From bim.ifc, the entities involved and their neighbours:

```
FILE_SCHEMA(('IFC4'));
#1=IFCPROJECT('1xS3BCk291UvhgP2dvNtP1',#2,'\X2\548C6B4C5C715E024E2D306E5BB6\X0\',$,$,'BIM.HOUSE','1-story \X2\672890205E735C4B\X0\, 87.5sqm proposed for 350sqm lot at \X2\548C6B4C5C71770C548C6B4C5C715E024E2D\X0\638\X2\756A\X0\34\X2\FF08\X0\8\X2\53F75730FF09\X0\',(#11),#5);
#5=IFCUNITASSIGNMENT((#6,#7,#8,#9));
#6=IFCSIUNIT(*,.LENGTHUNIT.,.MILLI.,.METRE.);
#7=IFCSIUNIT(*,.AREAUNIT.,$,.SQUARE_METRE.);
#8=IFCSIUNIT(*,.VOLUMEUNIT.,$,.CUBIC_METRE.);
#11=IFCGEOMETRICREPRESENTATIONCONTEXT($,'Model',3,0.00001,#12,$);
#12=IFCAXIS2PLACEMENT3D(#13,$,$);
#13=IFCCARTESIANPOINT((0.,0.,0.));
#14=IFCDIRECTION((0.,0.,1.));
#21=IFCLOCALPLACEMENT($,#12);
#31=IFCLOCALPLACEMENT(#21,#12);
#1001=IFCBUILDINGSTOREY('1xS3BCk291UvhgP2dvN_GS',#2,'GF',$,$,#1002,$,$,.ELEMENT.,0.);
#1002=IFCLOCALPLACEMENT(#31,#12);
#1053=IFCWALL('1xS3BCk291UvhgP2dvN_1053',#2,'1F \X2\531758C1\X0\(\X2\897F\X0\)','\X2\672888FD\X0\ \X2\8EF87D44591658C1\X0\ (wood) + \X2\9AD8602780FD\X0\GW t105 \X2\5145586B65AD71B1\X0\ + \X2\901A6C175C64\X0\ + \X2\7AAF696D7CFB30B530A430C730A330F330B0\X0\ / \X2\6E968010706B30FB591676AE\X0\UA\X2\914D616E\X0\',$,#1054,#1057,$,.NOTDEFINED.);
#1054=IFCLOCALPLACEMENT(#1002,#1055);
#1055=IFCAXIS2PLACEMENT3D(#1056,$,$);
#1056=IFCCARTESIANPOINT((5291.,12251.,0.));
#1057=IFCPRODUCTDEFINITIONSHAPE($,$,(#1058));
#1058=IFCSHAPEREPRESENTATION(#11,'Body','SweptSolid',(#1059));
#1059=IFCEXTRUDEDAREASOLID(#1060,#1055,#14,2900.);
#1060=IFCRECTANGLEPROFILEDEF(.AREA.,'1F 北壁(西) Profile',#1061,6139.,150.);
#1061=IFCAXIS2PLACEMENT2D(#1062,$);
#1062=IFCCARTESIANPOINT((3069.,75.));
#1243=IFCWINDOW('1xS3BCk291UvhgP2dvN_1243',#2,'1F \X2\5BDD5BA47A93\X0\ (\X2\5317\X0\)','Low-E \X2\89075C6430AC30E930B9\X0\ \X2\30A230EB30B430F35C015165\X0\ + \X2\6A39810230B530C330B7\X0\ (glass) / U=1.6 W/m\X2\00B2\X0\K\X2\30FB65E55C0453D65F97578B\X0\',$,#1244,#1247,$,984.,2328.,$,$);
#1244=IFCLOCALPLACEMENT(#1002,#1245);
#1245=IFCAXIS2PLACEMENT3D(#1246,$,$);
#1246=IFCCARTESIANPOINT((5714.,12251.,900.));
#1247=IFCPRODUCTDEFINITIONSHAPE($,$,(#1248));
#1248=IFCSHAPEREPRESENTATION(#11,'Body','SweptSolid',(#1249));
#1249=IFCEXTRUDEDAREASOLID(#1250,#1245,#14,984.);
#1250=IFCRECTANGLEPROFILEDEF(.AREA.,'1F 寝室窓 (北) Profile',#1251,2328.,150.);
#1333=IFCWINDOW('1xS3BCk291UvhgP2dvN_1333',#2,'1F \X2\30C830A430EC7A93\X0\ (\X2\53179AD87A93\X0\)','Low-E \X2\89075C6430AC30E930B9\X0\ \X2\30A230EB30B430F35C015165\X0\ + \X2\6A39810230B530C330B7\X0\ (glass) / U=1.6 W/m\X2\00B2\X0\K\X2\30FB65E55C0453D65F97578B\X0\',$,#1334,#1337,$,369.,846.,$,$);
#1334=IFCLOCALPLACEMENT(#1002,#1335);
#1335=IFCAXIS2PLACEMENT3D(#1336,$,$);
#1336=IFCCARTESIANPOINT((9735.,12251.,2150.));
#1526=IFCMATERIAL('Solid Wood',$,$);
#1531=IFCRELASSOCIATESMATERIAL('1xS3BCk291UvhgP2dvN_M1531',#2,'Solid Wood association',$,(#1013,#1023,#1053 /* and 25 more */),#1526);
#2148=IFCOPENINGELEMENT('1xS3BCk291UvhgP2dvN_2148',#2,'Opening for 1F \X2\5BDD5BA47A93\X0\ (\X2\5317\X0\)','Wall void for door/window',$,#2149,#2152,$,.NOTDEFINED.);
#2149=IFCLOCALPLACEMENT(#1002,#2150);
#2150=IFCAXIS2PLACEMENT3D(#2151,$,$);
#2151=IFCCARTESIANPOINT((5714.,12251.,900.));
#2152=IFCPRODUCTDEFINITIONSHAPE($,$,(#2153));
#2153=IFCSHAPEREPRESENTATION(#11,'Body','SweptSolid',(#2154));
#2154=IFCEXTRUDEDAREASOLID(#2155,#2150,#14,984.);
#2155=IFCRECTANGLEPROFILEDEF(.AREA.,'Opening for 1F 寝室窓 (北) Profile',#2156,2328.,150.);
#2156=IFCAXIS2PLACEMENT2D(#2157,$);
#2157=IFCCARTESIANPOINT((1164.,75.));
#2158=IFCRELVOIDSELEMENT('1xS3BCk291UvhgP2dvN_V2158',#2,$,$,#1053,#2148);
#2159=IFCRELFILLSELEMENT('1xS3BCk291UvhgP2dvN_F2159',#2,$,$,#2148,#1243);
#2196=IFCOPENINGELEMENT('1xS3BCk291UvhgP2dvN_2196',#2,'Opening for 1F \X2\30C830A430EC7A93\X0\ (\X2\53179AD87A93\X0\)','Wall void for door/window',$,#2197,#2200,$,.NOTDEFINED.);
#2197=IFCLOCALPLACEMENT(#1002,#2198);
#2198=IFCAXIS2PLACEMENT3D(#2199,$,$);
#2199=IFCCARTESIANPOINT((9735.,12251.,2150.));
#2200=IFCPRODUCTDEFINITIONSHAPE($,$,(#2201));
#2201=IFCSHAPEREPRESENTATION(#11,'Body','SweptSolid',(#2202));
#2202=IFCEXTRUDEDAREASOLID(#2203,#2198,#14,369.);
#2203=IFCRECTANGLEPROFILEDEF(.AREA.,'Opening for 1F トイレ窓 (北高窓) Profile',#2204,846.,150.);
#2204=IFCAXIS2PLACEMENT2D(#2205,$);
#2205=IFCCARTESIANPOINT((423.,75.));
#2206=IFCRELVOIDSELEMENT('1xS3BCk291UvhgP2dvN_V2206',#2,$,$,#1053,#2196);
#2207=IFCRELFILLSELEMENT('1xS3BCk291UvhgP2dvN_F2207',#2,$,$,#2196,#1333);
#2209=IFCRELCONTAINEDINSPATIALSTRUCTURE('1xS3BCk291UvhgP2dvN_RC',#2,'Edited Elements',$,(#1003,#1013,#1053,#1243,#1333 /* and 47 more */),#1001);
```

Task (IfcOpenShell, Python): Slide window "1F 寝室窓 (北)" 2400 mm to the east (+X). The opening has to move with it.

```python
import ifcopenshell
import ifcopenshell.api.geometry
import ifcopenshell.util.placement
import ifcopenshell.util.unit

model = ifcopenshell.open("bim.ifc")
unit_scale = ifcopenshell.util.unit.calculate_unit_scale(model)

window = model.by_id(1243)
opening = window.FillsVoids[0].RelatingOpeningElement
wall = opening.VoidsElements[0].RelatingBuildingElement

wall_matrix = ifcopenshell.util.placement.get_local_placement(wall.ObjectPlacement)
shift = wall_matrix[:3, 0] * 2.4 / unit_scale
before = ifcopenshell.util.placement.get_local_placement(window.ObjectPlacement)[:3, 3].copy()

# The window is not placed relative to its opening, so move both.
for product in (opening, window):
    matrix = ifcopenshell.util.placement.get_local_placement(product.ObjectPlacement)
    matrix[:3, 3] += shift
    ifcopenshell.api.geometry.edit_object_placement(model, product=product, matrix=matrix, is_si=False)

after = ifcopenshell.util.placement.get_local_placement(window.ObjectPlacement)[:3, 3]
print("window moved by", (after - before).round(3) + 0.0)

model.write("bim_rev.ifc")
```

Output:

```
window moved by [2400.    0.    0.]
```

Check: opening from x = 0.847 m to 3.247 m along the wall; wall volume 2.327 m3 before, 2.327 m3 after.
